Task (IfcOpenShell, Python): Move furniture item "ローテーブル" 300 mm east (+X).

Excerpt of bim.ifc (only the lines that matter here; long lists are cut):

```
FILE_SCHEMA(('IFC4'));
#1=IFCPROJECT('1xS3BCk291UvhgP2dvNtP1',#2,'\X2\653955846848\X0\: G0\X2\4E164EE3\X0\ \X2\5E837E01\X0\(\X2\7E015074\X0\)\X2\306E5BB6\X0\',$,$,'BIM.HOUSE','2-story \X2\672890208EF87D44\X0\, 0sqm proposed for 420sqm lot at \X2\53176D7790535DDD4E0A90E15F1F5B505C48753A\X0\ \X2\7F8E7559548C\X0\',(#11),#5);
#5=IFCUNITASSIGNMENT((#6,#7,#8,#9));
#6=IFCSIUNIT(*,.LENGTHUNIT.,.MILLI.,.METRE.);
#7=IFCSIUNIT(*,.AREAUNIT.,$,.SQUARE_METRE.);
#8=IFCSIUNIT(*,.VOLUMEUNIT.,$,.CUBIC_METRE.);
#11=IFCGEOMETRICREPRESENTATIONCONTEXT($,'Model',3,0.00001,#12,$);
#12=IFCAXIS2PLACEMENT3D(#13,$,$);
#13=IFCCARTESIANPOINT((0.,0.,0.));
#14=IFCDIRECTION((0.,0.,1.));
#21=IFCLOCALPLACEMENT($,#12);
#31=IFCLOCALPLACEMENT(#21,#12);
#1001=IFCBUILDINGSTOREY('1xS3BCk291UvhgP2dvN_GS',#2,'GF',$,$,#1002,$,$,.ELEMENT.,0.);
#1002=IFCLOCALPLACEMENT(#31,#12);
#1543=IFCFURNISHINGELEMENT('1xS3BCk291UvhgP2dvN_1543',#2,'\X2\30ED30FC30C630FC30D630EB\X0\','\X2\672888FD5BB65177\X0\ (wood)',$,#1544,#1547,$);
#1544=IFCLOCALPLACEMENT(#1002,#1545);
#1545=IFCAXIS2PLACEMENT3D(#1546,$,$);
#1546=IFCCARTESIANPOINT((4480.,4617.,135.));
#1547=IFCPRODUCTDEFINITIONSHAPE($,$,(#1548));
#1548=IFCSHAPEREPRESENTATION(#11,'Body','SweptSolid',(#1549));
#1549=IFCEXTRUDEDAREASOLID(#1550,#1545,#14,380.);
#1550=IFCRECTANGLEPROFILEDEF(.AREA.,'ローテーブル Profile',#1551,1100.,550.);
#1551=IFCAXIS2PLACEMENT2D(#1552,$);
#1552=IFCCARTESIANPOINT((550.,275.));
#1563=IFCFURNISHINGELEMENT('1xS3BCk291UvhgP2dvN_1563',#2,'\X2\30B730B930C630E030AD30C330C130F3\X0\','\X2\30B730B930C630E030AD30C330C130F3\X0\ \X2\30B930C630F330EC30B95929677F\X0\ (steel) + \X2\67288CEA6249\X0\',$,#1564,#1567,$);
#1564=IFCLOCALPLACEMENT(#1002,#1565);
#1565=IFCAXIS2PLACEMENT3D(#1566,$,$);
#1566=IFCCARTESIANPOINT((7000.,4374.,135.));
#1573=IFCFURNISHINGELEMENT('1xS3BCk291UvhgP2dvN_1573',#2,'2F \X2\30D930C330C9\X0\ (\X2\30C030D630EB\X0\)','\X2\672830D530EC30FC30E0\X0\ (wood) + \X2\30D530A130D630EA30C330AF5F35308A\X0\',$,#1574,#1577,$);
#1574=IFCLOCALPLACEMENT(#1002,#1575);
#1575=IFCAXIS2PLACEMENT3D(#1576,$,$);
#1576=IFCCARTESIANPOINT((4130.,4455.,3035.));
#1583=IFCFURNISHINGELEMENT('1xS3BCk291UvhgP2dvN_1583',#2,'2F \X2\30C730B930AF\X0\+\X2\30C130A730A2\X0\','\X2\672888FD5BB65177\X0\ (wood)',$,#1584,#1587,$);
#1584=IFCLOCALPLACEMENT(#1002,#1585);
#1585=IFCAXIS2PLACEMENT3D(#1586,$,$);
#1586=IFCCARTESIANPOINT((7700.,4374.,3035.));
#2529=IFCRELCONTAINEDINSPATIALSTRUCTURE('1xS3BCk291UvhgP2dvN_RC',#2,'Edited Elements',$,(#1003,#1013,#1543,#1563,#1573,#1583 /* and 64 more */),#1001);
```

```python
import ifcopenshell
import ifcopenshell.api.geometry
import ifcopenshell.util.placement
import ifcopenshell.util.unit

model = ifcopenshell.open("bim.ifc")
unit_scale = ifcopenshell.util.unit.calculate_unit_scale(model)

item = model.by_guid("1xS3BCk291UvhgP2dvN_1543")
matrix = ifcopenshell.util.placement.get_local_placement(item.ObjectPlacement)
matrix[0, 3] += 0.3 / unit_scale
ifcopenshell.api.geometry.edit_object_placement(model, product=item, matrix=matrix, is_si=False)

print(ifcopenshell.util.placement.get_local_placement(item.ObjectPlacement).round(3) + 0.0)

model.write("bim-out.ifc")
```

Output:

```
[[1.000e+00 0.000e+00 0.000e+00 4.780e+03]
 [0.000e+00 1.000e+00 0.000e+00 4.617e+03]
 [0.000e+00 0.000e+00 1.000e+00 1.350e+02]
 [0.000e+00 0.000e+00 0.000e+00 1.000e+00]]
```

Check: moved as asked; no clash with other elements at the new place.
